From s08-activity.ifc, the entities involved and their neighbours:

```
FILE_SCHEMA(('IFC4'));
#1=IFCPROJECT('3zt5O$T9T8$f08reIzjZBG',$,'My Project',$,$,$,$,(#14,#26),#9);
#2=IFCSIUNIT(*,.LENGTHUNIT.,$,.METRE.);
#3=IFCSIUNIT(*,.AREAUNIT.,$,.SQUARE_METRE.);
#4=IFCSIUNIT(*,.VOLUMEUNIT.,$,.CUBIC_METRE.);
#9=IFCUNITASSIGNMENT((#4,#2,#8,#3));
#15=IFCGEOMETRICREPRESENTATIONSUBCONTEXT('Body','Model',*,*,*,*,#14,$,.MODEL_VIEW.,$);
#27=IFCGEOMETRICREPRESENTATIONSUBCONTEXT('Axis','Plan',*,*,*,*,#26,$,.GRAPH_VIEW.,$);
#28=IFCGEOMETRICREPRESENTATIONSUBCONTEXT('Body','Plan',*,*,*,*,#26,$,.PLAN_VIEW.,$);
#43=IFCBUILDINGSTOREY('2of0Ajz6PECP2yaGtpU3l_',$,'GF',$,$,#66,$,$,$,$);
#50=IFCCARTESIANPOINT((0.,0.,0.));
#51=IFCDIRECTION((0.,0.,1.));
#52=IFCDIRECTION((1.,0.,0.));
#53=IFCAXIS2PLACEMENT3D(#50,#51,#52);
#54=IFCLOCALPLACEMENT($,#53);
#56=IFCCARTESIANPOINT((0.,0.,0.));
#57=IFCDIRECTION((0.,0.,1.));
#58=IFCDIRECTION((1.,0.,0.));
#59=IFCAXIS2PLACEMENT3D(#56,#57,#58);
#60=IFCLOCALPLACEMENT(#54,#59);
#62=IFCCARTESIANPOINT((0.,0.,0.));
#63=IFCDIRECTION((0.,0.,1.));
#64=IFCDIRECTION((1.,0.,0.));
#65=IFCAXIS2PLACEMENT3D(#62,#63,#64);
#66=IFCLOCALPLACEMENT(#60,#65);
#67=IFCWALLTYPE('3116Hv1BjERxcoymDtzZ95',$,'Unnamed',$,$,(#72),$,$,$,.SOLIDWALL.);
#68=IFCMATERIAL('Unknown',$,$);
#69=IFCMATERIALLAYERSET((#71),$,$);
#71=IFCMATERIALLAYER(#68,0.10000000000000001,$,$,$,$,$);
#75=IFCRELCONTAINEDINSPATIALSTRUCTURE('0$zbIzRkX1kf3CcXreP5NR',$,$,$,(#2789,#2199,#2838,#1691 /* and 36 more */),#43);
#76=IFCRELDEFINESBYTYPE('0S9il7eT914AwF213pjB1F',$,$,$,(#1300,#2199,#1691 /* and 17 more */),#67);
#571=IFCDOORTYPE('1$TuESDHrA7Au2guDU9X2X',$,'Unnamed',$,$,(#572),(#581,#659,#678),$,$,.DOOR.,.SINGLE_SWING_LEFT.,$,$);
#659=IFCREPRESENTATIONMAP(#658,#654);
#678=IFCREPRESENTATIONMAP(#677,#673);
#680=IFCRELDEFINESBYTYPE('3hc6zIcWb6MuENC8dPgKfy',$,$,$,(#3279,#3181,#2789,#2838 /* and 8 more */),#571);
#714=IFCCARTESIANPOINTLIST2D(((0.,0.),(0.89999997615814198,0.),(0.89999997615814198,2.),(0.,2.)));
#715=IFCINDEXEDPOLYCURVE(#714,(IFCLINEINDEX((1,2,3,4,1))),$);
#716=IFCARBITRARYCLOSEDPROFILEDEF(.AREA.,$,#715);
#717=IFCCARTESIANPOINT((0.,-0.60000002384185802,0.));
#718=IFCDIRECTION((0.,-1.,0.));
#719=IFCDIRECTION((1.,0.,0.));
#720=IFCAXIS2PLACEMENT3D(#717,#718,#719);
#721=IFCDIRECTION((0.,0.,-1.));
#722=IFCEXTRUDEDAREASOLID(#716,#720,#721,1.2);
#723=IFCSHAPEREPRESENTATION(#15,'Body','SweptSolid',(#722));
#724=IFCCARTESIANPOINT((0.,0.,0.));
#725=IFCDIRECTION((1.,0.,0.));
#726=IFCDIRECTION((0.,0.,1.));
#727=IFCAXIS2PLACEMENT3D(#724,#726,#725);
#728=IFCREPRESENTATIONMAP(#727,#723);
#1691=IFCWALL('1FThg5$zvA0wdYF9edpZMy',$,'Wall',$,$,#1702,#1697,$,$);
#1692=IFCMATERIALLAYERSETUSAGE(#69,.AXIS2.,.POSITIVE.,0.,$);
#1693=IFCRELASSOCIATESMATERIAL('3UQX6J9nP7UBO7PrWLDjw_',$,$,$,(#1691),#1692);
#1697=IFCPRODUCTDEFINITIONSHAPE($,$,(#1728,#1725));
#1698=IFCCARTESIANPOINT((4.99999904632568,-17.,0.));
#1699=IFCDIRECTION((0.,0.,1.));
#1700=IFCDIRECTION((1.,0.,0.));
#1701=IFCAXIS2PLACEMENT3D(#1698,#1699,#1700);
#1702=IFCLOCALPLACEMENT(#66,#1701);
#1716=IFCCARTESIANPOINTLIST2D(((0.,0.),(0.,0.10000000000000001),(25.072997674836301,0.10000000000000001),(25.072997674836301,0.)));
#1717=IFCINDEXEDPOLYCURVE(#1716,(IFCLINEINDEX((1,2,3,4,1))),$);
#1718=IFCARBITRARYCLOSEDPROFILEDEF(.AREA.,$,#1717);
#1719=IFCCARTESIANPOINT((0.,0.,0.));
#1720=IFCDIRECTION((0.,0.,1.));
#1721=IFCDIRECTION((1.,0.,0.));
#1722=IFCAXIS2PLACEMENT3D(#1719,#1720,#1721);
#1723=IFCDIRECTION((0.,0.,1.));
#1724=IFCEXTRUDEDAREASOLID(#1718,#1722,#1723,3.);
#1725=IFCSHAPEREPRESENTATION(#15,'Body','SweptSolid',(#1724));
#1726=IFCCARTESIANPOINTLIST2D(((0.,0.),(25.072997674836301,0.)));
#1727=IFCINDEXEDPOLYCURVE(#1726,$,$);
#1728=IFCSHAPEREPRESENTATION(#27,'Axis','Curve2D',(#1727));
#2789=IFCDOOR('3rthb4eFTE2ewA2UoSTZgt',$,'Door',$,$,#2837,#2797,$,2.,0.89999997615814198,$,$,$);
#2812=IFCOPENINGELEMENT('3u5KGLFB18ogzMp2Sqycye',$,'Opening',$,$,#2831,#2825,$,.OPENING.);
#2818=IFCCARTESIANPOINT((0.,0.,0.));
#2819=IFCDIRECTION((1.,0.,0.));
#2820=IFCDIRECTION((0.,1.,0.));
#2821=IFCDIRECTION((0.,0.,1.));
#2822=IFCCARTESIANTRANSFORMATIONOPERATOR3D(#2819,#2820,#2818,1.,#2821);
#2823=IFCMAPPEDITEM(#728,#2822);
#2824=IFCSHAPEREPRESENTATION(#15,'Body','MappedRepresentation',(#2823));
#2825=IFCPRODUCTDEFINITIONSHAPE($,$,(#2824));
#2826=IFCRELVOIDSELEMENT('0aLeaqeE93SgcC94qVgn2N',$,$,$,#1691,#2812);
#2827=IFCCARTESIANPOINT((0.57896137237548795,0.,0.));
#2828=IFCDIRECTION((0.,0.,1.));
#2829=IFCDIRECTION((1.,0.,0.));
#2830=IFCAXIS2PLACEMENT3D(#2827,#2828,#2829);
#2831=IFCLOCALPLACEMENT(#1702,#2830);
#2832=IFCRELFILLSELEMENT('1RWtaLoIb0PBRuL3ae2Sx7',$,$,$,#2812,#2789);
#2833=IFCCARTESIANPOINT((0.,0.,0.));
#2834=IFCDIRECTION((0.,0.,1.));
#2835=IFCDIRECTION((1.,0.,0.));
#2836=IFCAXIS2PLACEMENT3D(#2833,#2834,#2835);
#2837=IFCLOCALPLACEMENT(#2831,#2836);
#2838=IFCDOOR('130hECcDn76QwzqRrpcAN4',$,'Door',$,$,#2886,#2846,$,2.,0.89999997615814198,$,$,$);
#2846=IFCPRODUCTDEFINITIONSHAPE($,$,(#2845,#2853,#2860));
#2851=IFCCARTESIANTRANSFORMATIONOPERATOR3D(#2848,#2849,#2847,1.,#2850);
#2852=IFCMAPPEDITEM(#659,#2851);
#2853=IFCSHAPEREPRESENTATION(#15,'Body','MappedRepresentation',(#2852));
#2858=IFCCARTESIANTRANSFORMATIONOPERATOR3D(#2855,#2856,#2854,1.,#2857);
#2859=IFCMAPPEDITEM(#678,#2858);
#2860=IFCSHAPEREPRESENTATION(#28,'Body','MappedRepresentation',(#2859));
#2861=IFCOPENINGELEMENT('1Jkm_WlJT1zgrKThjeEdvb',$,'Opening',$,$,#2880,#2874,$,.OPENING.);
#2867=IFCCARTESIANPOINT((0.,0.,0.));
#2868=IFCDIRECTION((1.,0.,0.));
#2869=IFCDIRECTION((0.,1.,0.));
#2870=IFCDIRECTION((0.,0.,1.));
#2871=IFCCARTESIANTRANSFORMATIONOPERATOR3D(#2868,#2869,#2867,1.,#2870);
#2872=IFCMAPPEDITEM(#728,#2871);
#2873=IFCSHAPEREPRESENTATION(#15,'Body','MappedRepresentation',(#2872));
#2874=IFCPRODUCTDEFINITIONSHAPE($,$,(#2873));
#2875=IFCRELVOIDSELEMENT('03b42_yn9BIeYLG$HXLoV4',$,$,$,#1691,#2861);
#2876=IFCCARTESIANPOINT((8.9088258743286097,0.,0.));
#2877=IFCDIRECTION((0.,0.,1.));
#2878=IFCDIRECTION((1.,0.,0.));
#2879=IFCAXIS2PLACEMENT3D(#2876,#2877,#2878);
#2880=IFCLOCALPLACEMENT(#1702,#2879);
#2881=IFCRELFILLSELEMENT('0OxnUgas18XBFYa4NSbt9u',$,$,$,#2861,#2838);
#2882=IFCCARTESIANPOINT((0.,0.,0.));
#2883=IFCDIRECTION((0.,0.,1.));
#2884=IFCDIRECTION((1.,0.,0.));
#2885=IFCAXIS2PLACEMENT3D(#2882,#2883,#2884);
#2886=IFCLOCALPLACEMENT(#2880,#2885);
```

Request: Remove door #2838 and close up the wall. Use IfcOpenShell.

```python
import ifcopenshell
import ifcopenshell.api.feature
import ifcopenshell.api.root
import ifcopenshell.geom
import ifcopenshell.util.shape

model = ifcopenshell.open("s08-activity.ifc")
settings = ifcopenshell.geom.settings()


def volume(element):
    """Net volume in cubic metres, openings subtracted."""
    shape = ifcopenshell.geom.create_shape(settings, element)
    return ifcopenshell.util.shape.get_volume(shape.geometry)


door = model.by_guid("130hECcDn76QwzqRrpcAN4")
opening = door.FillsVoids[0].RelatingOpeningElement
wall = opening.VoidsElements[0].RelatingBuildingElement
before = volume(wall)

ifcopenshell.api.root.remove_product(model, product=door)
ifcopenshell.api.feature.remove_feature(model, feature=opening)

after = volume(wall)

print(f"wall volume {before:.3f} -> {after:.3f} m3")

model.write("s08-activity_edited.ifc")
```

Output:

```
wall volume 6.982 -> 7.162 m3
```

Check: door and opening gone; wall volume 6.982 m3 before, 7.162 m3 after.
